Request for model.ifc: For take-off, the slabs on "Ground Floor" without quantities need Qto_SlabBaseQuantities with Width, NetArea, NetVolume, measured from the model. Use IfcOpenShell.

First a look at what the model holds.

```python
import ifcopenshell
import ifcopenshell.util.element
import ifcopenshell.util.unit

model = ifcopenshell.open("model.ifc")
print(model.schema)
for unit_type in ("LENGTHUNIT", "AREAUNIT", "VOLUMEUNIT"):
    print(unit_type, ifcopenshell.util.unit.calculate_unit_scale(model, unit_type))
storey = next(s for s in model.by_type("IfcBuildingStorey") if s.Name == "Ground Floor")
slabs = [e for e in ifcopenshell.util.element.get_decomposition(storey) if e.is_a("IfcSlab")]
for e in sorted(slabs, key=lambda e: e.id()):
    print(e.id(), e.is_a(), e.Name, list(ifcopenshell.util.element.get_psets(e, qtos_only=True)), sep=" | ")
```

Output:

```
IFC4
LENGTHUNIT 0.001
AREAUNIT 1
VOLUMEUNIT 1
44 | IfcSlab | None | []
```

```python
import ifcopenshell
import ifcopenshell.api.pset
import ifcopenshell.geom
import ifcopenshell.util.element
import ifcopenshell.util.shape
import ifcopenshell.util.unit

model = ifcopenshell.open("model.ifc")
unit_scale = ifcopenshell.util.unit.calculate_unit_scale(model)
area_scale = ifcopenshell.util.unit.calculate_unit_scale(model, "AREAUNIT")
volume_scale = ifcopenshell.util.unit.calculate_unit_scale(model, "VOLUMEUNIT")
settings = ifcopenshell.geom.settings()

storey = next(s for s in model.by_type("IfcBuildingStorey") if s.Name == "Ground Floor")
slabs = [e for e in ifcopenshell.util.element.get_decomposition(storey) if e.is_a("IfcSlab")]

for e in sorted(slabs, key=lambda e: e.id()):
    if ifcopenshell.util.element.get_psets(e, qtos_only=True, should_inherit=False):
        continue
    # Geometry comes back in metres, in the element's own axes.
    shape = ifcopenshell.geom.create_shape(settings, e)
    values = {
        "Width": ifcopenshell.util.shape.get_z(shape.geometry) / unit_scale,
        "NetArea": ifcopenshell.util.shape.get_footprint_area(shape.geometry) / area_scale,
        "NetVolume": ifcopenshell.util.shape.get_volume(shape.geometry) / volume_scale,
    }
    qto = ifcopenshell.api.pset.add_qto(model, product=e, name="Qto_SlabBaseQuantities")
    ifcopenshell.api.pset.edit_qto(model, qto=qto, properties=values)
    print(e.id(), {k: round(v, 3) for k, v in values.items()})

model.write("model_edited.ifc")
```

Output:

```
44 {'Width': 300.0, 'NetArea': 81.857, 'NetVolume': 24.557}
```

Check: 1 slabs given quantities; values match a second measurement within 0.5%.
